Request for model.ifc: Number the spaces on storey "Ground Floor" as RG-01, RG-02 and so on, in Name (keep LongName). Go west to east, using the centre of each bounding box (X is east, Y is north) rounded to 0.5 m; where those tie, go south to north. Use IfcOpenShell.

First a look at what the model holds.

```python
import ifcopenshell
import ifcopenshell.util.element
import ifcopenshell.util.placement

model = ifcopenshell.open("model.ifc")
print(model.schema)
storey = next(s for s in model.by_type("IfcBuildingStorey") if s.Name == "Ground Floor")
spaces = [e for e in ifcopenshell.util.element.get_decomposition(storey) if e.is_a("IfcSpace")]
for e in sorted(spaces, key=lambda e: e.id()):
    origin = ifcopenshell.util.placement.get_local_placement(e.ObjectPlacement)[:3, 3]
    print(e.id(), e.Name, e.LongName, origin.round(2) + 0.0, sep=" | ")
```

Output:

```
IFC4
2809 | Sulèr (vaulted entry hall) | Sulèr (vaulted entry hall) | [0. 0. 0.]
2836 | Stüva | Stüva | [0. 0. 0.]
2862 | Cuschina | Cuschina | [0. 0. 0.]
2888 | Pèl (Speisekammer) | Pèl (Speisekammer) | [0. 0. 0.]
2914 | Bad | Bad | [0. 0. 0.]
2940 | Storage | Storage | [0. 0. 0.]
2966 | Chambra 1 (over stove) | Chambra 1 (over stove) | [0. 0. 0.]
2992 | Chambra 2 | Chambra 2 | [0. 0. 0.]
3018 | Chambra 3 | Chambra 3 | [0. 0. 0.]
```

```python
import ifcopenshell
import ifcopenshell.geom
import ifcopenshell.util.element
import ifcopenshell.util.shape

model = ifcopenshell.open("model.ifc")
settings = ifcopenshell.geom.settings()
settings.set("use-world-coords", True)


def centre(element):
    shape = ifcopenshell.geom.create_shape(settings, element)
    return ifcopenshell.util.shape.get_bbox_centroid(shape.geometry)


storey = next(s for s in model.by_type("IfcBuildingStorey") if s.Name == "Ground Floor")
spaces = [e for e in ifcopenshell.util.element.get_decomposition(storey) if e.is_a("IfcSpace")]

# Insertion points can sit at a corner or the storey origin, so sort by the geometry (in metres).
centres = {e: centre(e) for e in spaces}
spaces.sort(key=lambda e: (round(centres[e][0] / 0.5), centres[e][1]))

for i, e in enumerate(spaces, start=1):
    number = f"RG-{i:02d}"
    e.Name = number
    print(e.id(), number)

model.write("model_rev.ifc")
```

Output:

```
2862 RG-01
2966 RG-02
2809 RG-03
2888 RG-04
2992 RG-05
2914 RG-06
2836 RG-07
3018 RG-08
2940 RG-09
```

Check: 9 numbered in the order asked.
